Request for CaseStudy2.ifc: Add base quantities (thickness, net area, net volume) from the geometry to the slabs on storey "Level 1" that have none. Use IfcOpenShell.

First a look at what the model holds.

```python
import ifcopenshell
import ifcopenshell.util.element
import ifcopenshell.util.unit

model = ifcopenshell.open("CaseStudy2.ifc")
print(model.schema)
for unit_type in ("LENGTHUNIT", "AREAUNIT", "VOLUMEUNIT"):
    print(unit_type, ifcopenshell.util.unit.calculate_unit_scale(model, unit_type))
storey = next(s for s in model.by_type("IfcBuildingStorey") if s.Name == "Level 1")
slabs = [e for e in ifcopenshell.util.element.get_decomposition(storey) if e.is_a("IfcSlab")]
for e in sorted(slabs, key=lambda e: e.id()):
    print(e.id(), e.is_a(), e.Name, list(ifcopenshell.util.element.get_psets(e, qtos_only=True)), sep=" | ")
```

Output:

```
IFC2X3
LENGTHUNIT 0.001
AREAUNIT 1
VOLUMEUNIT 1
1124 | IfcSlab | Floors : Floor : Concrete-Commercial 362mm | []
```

```python
import ifcopenshell
import ifcopenshell.api.pset
import ifcopenshell.geom
import ifcopenshell.util.element
import ifcopenshell.util.shape
import ifcopenshell.util.unit

model = ifcopenshell.open("CaseStudy2.ifc")
unit_scale = ifcopenshell.util.unit.calculate_unit_scale(model)
area_scale = ifcopenshell.util.unit.calculate_unit_scale(model, "AREAUNIT")
volume_scale = ifcopenshell.util.unit.calculate_unit_scale(model, "VOLUMEUNIT")
settings = ifcopenshell.geom.settings()

storey = next(s for s in model.by_type("IfcBuildingStorey") if s.Name == "Level 1")
slabs = [e for e in ifcopenshell.util.element.get_decomposition(storey) if e.is_a("IfcSlab")]

for e in sorted(slabs, key=lambda e: e.id()):
    if ifcopenshell.util.element.get_psets(e, qtos_only=True, should_inherit=False):
        continue
    # Geometry comes back in metres, in the element's own axes.
    shape = ifcopenshell.geom.create_shape(settings, e)
    values = {
        "Width": ifcopenshell.util.shape.get_z(shape.geometry) / unit_scale,
        "NetArea": ifcopenshell.util.shape.get_footprint_area(shape.geometry) / area_scale,
        "NetVolume": ifcopenshell.util.shape.get_volume(shape.geometry) / volume_scale,
    }
    qto = ifcopenshell.api.pset.add_qto(model, product=e, name="BaseQuantities")
    ifcopenshell.api.pset.edit_qto(model, qto=qto, properties=values)
    print(e.id(), {k: round(v, 3) for k, v in values.items()})

model.write("CaseStudy2_v2.ifc")
```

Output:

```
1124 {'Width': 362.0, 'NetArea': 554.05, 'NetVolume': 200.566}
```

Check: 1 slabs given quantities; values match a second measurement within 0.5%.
